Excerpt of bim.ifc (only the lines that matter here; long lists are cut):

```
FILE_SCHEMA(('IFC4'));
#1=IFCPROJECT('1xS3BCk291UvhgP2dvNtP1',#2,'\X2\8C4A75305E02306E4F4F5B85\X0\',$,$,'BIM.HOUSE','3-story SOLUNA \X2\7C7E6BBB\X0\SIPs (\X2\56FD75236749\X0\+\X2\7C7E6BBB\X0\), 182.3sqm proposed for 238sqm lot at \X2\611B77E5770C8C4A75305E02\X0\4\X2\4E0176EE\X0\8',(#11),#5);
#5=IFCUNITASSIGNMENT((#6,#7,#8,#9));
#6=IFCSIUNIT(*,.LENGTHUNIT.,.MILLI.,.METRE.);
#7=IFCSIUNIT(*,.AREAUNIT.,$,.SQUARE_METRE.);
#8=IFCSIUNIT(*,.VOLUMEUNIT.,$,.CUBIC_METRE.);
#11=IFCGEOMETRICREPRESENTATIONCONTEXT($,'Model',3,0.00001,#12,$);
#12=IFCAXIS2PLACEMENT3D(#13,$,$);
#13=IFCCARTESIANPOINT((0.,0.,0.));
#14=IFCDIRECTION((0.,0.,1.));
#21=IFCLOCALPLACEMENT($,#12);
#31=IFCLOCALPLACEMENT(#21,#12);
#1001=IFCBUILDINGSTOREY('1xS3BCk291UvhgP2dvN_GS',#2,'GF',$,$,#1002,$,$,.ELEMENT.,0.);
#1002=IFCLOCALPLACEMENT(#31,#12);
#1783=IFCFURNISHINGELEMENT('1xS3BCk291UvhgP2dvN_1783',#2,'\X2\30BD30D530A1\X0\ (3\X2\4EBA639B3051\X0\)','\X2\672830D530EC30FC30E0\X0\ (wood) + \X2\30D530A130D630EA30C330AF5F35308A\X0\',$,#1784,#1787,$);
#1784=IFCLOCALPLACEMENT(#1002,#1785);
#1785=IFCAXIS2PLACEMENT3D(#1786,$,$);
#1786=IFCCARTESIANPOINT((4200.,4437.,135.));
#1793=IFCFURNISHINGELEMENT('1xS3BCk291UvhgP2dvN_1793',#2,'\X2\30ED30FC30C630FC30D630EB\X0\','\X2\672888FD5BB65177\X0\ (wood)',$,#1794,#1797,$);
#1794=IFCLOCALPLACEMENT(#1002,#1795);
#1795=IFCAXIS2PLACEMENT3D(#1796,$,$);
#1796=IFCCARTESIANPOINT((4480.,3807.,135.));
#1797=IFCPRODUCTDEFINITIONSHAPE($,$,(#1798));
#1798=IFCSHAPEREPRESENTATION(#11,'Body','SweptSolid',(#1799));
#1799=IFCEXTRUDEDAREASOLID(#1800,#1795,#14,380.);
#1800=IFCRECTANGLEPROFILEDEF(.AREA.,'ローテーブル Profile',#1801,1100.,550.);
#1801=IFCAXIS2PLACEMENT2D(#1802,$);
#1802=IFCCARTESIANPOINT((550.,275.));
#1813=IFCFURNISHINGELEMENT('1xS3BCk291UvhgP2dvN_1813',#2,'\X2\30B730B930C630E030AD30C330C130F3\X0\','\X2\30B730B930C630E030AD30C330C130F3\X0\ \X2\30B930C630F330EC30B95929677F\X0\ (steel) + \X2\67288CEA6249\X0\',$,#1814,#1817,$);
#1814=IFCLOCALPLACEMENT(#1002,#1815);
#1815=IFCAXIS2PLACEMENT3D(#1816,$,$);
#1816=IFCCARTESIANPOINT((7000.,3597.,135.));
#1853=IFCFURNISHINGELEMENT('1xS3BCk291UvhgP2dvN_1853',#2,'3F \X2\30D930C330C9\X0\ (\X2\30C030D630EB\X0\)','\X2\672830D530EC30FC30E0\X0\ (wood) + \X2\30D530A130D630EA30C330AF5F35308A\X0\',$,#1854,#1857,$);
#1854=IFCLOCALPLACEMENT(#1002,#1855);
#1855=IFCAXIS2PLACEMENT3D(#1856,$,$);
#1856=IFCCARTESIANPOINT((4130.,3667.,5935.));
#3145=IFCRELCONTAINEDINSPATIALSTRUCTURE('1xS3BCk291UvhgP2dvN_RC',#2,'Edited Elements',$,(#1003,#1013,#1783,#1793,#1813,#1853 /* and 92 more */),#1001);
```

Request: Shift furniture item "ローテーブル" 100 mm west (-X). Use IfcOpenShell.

```python
import ifcopenshell
import ifcopenshell.api.geometry
import ifcopenshell.util.placement
import ifcopenshell.util.unit

model = ifcopenshell.open("bim.ifc")
unit_scale = ifcopenshell.util.unit.calculate_unit_scale(model)

item = model.by_guid("1xS3BCk291UvhgP2dvN_1793")
matrix = ifcopenshell.util.placement.get_local_placement(item.ObjectPlacement)
matrix[0, 3] -= 0.1 / unit_scale
ifcopenshell.api.geometry.edit_object_placement(model, product=item, matrix=matrix, is_si=False)

print(ifcopenshell.util.placement.get_local_placement(item.ObjectPlacement).round(3) + 0.0)

model.write("bim_v2.ifc")
```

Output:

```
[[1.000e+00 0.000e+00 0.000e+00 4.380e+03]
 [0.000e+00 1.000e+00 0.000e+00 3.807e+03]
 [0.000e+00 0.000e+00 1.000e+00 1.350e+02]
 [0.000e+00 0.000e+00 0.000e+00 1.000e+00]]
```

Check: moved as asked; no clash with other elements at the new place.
